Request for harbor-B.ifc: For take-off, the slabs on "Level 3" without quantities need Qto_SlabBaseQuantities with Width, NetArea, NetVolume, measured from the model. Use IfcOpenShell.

First a look at what the model holds.

```python
import ifcopenshell
import ifcopenshell.util.element
import ifcopenshell.util.unit

model = ifcopenshell.open("harbor-B.ifc")
print(model.schema)
for unit_type in ("LENGTHUNIT", "AREAUNIT", "VOLUMEUNIT"):
    print(unit_type, ifcopenshell.util.unit.calculate_unit_scale(model, unit_type))
storey = next(s for s in model.by_type("IfcBuildingStorey") if s.Name == "Level 3")
slabs = [e for e in ifcopenshell.util.element.get_decomposition(storey) if e.is_a("IfcSlab")]
for e in sorted(slabs, key=lambda e: e.id()):
    print(e.id(), e.is_a(), e.Name, list(ifcopenshell.util.element.get_psets(e, qtos_only=True)), sep=" | ")
```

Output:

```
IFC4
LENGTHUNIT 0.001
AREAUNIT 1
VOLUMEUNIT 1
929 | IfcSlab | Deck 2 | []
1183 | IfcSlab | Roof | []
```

```python
import ifcopenshell
import ifcopenshell.api.pset
import ifcopenshell.geom
import ifcopenshell.util.element
import ifcopenshell.util.shape
import ifcopenshell.util.unit

model = ifcopenshell.open("harbor-B.ifc")
unit_scale = ifcopenshell.util.unit.calculate_unit_scale(model)
area_scale = ifcopenshell.util.unit.calculate_unit_scale(model, "AREAUNIT")
volume_scale = ifcopenshell.util.unit.calculate_unit_scale(model, "VOLUMEUNIT")
settings = ifcopenshell.geom.settings()

storey = next(s for s in model.by_type("IfcBuildingStorey") if s.Name == "Level 3")
slabs = [e for e in ifcopenshell.util.element.get_decomposition(storey) if e.is_a("IfcSlab")]

for e in sorted(slabs, key=lambda e: e.id()):
    if ifcopenshell.util.element.get_psets(e, qtos_only=True, should_inherit=False):
        continue
    # Geometry comes back in metres, in the element's own axes.
    shape = ifcopenshell.geom.create_shape(settings, e)
    values = {
        "Width": ifcopenshell.util.shape.get_z(shape.geometry) / unit_scale,
        "NetArea": ifcopenshell.util.shape.get_footprint_area(shape.geometry) / area_scale,
        "NetVolume": ifcopenshell.util.shape.get_volume(shape.geometry) / volume_scale,
    }
    qto = ifcopenshell.api.pset.add_qto(model, product=e, name="Qto_SlabBaseQuantities")
    ifcopenshell.api.pset.edit_qto(model, qto=qto, properties=values)
    print(e.id(), {k: round(v, 3) for k, v in values.items()})

model.write("harbor-B_updated.ifc")
```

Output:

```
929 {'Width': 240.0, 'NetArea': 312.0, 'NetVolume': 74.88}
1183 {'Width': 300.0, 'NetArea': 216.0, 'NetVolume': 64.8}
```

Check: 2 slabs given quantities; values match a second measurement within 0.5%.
